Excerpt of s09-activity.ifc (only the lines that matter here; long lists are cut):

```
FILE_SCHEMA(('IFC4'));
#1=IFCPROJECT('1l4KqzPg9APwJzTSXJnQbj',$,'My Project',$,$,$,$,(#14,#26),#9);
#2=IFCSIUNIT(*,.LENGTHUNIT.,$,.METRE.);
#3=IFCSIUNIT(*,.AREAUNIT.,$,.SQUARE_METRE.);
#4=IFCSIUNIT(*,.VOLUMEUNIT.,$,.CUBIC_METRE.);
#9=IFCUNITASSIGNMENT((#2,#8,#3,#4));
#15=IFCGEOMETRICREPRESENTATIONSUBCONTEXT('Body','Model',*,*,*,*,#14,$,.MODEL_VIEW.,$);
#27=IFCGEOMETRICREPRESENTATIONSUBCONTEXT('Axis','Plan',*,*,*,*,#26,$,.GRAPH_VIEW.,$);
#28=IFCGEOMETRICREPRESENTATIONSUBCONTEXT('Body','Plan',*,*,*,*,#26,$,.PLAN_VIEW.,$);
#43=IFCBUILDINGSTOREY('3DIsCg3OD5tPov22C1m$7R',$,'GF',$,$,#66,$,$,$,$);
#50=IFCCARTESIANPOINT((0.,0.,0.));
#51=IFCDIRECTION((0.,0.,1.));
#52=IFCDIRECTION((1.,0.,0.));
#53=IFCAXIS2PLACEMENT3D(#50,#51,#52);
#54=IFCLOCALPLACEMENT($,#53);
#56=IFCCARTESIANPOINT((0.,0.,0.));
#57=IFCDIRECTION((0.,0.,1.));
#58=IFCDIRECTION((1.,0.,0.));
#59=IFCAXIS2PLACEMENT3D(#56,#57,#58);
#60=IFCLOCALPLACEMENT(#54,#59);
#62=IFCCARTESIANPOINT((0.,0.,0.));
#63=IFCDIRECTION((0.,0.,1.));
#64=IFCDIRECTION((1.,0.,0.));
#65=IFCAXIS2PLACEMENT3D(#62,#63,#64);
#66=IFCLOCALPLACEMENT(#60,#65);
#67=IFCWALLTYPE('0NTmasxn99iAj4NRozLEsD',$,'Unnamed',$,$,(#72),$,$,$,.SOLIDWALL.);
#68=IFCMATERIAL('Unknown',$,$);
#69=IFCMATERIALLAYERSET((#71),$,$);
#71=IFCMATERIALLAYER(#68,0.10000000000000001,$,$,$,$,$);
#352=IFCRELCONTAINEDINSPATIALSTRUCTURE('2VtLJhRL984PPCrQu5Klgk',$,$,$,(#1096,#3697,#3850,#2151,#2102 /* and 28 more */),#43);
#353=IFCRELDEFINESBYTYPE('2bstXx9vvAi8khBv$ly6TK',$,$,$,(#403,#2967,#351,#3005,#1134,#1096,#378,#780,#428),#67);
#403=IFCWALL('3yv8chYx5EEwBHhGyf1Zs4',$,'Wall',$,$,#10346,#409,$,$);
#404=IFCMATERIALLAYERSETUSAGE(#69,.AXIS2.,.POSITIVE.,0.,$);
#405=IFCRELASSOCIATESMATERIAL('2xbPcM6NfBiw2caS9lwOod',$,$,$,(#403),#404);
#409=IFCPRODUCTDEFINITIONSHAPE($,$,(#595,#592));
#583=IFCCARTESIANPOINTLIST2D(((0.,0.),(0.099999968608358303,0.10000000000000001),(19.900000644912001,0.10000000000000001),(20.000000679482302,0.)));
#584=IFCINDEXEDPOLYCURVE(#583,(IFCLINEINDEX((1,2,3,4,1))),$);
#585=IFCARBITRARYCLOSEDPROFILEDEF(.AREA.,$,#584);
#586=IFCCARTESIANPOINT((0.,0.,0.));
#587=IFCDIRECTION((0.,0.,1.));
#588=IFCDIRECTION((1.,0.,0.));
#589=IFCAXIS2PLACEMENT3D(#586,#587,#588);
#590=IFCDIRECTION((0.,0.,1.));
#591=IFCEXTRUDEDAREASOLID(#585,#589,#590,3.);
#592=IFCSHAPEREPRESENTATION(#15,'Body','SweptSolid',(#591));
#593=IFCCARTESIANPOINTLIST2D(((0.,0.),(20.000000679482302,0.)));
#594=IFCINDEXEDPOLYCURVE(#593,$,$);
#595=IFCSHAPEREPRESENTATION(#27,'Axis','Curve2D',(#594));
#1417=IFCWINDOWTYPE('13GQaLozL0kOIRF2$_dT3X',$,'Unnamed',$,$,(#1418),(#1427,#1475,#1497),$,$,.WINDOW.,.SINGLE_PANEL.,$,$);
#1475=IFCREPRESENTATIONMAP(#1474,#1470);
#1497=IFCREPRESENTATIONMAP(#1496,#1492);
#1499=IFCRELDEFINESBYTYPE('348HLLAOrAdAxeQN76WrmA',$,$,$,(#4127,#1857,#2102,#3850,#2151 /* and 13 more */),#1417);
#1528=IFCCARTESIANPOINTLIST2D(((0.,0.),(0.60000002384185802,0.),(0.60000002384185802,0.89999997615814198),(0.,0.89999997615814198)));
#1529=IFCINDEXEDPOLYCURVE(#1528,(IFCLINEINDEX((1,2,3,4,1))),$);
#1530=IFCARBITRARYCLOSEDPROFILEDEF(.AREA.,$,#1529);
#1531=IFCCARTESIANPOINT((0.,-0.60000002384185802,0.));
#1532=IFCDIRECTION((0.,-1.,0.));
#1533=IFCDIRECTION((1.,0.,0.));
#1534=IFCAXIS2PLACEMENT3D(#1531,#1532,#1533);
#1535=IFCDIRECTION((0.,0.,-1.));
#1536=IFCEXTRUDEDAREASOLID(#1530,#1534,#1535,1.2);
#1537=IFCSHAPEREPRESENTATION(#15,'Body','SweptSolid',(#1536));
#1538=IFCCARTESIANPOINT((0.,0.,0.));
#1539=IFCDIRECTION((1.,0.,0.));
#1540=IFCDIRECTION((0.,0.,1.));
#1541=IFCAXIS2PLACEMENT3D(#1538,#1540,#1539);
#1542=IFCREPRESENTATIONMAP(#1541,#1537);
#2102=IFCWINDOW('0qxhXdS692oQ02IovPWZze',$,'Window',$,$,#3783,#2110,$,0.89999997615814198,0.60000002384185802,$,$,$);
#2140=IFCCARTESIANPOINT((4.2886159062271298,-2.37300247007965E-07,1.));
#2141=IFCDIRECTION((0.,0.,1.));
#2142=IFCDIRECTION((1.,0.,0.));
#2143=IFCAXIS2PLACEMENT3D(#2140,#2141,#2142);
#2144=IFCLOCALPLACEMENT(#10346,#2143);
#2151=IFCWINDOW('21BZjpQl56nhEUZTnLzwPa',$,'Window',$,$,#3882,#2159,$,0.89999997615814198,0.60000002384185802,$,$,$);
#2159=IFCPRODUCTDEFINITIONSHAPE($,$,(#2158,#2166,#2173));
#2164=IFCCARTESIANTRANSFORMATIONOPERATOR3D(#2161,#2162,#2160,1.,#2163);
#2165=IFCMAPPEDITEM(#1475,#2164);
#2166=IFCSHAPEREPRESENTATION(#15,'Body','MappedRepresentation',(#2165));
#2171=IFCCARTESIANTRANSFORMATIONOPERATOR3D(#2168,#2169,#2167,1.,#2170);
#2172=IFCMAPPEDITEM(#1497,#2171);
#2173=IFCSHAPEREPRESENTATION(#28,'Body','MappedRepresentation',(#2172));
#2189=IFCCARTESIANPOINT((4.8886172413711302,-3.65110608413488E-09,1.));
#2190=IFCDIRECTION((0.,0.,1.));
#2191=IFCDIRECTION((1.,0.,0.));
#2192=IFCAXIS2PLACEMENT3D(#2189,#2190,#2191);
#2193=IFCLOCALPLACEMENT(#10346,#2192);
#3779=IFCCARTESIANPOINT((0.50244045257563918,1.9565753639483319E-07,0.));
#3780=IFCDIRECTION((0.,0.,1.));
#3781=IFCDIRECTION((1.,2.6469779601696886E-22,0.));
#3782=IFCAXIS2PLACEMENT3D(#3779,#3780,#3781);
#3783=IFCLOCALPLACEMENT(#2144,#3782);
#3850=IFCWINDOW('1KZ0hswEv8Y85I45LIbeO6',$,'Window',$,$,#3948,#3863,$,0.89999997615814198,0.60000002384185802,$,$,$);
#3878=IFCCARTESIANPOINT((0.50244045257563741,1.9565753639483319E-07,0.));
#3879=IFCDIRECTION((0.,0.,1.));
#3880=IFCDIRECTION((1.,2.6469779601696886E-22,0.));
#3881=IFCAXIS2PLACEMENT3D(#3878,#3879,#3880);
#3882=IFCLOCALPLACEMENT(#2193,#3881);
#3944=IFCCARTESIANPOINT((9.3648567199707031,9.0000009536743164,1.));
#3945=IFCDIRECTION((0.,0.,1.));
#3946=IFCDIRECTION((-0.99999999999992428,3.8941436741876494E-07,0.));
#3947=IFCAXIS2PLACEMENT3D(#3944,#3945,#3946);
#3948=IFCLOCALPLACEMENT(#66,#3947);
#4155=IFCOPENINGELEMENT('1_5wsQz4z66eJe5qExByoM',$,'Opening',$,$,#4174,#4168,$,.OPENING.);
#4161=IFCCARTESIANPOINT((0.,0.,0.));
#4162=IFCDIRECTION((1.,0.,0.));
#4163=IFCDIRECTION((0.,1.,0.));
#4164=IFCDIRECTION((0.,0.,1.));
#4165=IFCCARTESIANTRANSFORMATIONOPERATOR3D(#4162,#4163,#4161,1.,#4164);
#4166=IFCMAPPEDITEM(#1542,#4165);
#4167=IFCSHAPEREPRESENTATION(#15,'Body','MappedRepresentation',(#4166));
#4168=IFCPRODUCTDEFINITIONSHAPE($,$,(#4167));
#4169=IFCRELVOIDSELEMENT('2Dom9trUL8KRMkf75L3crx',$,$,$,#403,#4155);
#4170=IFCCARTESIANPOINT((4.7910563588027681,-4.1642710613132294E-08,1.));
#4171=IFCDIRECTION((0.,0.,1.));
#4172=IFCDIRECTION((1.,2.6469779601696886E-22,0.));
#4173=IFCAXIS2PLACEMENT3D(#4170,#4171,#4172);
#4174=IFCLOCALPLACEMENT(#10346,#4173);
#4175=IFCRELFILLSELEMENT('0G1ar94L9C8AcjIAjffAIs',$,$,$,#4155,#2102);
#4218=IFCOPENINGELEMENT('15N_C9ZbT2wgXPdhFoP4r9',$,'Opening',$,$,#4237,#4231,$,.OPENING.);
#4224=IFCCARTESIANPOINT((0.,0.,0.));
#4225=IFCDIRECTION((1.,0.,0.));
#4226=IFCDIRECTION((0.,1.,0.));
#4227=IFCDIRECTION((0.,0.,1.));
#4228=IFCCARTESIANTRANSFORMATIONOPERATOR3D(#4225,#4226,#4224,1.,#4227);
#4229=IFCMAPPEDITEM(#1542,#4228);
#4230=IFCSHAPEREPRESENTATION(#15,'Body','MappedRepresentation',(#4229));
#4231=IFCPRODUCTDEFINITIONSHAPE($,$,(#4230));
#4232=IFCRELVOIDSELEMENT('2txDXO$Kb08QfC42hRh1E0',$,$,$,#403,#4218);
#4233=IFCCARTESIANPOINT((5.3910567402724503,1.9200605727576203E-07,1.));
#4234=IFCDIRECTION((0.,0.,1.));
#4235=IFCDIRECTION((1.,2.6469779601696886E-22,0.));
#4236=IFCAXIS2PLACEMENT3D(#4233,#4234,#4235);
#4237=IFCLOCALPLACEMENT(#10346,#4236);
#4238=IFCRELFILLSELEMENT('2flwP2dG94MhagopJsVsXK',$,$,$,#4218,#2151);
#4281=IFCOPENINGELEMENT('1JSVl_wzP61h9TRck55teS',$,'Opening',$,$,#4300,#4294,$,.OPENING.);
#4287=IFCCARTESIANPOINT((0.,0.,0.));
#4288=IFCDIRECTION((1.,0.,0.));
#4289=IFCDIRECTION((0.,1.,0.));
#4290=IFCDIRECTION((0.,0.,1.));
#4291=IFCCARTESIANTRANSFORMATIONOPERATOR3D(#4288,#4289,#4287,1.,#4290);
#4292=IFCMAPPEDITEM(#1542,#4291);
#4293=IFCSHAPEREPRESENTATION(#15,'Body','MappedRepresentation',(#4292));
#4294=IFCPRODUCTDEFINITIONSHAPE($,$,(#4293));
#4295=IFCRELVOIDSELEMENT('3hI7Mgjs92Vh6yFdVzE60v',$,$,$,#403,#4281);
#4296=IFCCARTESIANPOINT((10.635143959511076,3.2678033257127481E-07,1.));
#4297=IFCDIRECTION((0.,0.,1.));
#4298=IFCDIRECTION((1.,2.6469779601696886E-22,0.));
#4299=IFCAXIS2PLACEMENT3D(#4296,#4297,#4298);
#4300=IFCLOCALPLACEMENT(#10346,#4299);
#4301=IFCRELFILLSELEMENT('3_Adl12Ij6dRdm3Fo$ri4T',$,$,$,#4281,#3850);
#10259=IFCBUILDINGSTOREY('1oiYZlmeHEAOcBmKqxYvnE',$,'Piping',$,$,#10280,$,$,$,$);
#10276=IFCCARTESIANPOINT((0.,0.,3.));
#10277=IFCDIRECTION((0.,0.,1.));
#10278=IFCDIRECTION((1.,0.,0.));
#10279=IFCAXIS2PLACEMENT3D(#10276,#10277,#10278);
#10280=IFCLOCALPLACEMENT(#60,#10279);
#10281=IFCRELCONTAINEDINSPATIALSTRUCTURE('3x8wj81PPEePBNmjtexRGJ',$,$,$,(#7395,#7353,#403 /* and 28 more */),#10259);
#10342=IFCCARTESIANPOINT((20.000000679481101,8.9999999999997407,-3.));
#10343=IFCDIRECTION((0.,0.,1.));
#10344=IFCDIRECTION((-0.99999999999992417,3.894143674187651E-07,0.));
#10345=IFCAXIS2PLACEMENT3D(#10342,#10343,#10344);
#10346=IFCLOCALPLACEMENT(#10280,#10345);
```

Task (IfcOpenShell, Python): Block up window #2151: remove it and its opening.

```python
import ifcopenshell
import ifcopenshell.api.feature
import ifcopenshell.api.root
import ifcopenshell.geom
import ifcopenshell.util.shape

model = ifcopenshell.open("s09-activity.ifc")
settings = ifcopenshell.geom.settings()


def volume(element):
    """Net volume in cubic metres, openings subtracted."""
    shape = ifcopenshell.geom.create_shape(settings, element)
    return ifcopenshell.util.shape.get_volume(shape.geometry)


window = model.by_id(2151)
opening = window.FillsVoids[0].RelatingOpeningElement
wall = opening.VoidsElements[0].RelatingBuildingElement
before = volume(wall)

ifcopenshell.api.root.remove_product(model, product=window)
ifcopenshell.api.feature.remove_feature(model, feature=opening)

after = volume(wall)

print(f"wall volume {before:.3f} -> {after:.3f} m3")

model.write("s09-activity_rev.ifc")
```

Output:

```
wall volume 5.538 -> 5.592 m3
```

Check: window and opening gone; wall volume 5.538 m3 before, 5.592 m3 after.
